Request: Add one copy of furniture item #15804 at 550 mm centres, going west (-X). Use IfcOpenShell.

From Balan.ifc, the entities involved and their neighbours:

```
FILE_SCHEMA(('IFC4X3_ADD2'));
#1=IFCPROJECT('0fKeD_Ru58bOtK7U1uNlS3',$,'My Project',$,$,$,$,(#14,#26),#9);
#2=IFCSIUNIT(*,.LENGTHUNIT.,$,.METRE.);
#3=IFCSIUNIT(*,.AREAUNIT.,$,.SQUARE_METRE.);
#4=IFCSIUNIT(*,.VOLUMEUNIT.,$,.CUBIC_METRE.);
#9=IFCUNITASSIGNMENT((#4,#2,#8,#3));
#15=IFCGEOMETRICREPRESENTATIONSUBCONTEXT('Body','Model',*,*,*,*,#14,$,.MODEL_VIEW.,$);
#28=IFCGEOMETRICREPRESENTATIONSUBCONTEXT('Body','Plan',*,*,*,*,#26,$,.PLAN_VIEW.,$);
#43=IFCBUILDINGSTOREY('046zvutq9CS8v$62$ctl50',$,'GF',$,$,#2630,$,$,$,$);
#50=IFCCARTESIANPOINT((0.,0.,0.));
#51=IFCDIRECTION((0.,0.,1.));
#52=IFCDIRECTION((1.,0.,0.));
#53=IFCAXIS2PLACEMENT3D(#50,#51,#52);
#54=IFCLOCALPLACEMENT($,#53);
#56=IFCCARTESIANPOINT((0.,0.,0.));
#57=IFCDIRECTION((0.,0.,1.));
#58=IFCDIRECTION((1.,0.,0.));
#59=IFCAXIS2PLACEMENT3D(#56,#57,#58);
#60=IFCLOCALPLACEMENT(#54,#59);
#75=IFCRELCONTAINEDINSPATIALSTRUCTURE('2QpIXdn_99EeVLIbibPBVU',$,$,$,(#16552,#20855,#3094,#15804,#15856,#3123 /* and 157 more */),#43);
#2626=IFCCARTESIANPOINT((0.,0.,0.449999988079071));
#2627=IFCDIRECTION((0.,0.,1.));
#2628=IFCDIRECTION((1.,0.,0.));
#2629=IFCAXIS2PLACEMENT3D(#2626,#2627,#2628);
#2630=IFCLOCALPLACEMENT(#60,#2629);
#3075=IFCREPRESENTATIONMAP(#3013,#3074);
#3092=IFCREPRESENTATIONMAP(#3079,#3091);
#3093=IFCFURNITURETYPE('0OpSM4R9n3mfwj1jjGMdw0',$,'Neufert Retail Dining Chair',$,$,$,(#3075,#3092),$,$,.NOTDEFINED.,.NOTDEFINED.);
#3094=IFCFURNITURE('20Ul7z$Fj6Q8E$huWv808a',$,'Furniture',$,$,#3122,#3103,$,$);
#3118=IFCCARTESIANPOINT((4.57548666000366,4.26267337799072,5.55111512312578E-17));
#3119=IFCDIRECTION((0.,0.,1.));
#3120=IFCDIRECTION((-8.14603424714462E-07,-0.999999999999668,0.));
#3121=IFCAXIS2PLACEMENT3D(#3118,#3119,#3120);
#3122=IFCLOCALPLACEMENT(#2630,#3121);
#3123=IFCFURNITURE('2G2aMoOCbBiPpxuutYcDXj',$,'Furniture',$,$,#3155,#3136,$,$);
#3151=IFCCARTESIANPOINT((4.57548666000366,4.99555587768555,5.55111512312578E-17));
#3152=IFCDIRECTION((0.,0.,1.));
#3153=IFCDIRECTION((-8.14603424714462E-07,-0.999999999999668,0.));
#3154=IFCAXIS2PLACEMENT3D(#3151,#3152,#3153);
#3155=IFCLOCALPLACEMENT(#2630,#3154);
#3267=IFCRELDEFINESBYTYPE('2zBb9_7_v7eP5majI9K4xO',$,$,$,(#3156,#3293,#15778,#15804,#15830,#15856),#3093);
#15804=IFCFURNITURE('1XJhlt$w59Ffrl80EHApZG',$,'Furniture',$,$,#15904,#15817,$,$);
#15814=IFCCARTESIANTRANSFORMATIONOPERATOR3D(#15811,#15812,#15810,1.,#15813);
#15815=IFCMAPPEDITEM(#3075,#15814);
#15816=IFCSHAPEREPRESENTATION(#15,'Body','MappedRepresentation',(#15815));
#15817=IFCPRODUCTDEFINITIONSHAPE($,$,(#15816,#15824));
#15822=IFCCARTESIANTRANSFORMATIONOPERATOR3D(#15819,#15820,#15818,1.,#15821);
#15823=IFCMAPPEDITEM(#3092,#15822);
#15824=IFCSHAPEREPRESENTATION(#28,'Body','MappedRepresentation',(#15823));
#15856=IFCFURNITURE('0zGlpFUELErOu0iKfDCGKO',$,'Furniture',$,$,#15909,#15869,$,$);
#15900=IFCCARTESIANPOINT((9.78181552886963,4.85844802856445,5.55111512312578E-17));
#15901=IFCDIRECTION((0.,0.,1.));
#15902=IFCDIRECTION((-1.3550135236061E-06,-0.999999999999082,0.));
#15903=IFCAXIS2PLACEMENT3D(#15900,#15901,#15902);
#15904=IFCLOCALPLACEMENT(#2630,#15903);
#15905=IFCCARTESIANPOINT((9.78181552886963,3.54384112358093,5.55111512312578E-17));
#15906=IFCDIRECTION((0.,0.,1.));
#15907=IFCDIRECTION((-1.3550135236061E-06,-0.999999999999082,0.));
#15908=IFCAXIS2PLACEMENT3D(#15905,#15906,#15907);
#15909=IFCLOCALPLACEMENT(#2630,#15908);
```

```python
import numpy as np
import ifcopenshell
import ifcopenshell.api.geometry
import ifcopenshell.api.root
import ifcopenshell.util.element
import ifcopenshell.util.placement
import ifcopenshell.util.unit

model = ifcopenshell.open("Balan.ifc")
unit_scale = ifcopenshell.util.unit.calculate_unit_scale(model)

source = model.by_guid("1XJhlt$w59Ffrl80EHApZG")
base = ifcopenshell.util.placement.get_local_placement(source.ObjectPlacement)
step = np.array([-1.0, 0.0, 0.0]) * 0.55 / unit_scale

for i in range(1, 2):
    copy = ifcopenshell.api.root.copy_class(model, product=source)
    copy.Representation = ifcopenshell.util.element.copy_deep(
        model, source.Representation, exclude=["IfcGeometricRepresentationContext", "IfcRepresentationMap"]
    )
    matrix = base.copy()
    matrix[:3, 3] += i * step
    print("added at", matrix[:3, 3].round(3) + 0.0)
    ifcopenshell.api.geometry.edit_object_placement(model, product=copy, matrix=matrix, is_si=False)

model.write("Balan_edited.ifc")
```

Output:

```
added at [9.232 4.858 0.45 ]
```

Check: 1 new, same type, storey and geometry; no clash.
